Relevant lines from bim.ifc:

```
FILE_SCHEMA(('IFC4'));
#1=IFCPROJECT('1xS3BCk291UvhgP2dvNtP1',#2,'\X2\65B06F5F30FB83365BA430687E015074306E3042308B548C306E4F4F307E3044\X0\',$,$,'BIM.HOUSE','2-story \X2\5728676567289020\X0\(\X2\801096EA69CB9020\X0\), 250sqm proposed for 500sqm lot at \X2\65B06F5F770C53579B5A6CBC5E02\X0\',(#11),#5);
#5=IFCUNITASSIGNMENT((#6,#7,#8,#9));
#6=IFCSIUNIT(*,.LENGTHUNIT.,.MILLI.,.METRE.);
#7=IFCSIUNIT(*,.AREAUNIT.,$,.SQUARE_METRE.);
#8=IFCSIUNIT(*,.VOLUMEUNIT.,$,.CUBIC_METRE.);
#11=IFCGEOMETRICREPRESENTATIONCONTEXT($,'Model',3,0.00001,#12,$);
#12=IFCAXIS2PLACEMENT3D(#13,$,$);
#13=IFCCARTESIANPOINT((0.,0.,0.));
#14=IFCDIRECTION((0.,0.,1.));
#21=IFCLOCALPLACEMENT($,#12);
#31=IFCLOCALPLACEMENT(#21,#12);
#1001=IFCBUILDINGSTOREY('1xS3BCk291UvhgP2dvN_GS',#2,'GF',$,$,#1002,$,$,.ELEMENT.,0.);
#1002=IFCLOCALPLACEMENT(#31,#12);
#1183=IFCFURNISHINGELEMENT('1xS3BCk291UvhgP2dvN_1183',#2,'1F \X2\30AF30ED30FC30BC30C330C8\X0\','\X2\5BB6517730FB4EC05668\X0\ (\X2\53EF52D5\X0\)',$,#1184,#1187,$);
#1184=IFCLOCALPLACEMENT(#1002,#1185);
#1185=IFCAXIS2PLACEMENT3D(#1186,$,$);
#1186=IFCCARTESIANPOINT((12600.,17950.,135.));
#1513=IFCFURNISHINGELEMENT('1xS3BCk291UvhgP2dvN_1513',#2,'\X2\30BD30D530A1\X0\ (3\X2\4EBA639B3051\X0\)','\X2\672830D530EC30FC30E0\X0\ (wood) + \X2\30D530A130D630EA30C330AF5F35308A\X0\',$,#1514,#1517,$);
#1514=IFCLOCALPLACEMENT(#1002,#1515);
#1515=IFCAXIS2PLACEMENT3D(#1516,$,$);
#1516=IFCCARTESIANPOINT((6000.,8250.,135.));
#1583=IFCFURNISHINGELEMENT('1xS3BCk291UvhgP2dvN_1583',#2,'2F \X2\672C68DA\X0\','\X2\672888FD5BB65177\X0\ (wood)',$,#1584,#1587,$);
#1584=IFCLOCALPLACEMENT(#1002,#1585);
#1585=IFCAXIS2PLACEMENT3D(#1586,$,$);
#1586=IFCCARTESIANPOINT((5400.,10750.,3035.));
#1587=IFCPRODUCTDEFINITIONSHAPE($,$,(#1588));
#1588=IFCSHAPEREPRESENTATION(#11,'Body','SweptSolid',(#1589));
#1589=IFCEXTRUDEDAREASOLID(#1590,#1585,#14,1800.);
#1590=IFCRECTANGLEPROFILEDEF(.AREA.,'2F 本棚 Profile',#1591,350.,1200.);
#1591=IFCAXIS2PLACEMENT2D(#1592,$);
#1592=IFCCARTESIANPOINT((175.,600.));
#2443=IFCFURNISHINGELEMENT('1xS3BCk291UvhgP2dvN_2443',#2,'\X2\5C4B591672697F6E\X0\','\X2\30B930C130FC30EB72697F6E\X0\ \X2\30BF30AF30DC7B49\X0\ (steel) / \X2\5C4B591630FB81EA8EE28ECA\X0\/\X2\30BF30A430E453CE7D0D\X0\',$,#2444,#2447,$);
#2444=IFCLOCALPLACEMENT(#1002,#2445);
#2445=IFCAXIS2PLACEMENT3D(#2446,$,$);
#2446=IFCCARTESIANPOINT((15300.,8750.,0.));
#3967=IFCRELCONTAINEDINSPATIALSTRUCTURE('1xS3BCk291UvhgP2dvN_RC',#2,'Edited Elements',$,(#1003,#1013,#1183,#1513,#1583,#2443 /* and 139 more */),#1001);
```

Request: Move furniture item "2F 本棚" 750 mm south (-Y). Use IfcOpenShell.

```python
import ifcopenshell
import ifcopenshell.api.geometry
import ifcopenshell.util.placement
import ifcopenshell.util.unit

model = ifcopenshell.open("bim.ifc")
unit_scale = ifcopenshell.util.unit.calculate_unit_scale(model)

item = model.by_guid("1xS3BCk291UvhgP2dvN_1583")
matrix = ifcopenshell.util.placement.get_local_placement(item.ObjectPlacement)
matrix[1, 3] -= 0.75 / unit_scale
ifcopenshell.api.geometry.edit_object_placement(model, product=item, matrix=matrix, is_si=False)

print(ifcopenshell.util.placement.get_local_placement(item.ObjectPlacement).round(3) + 0.0)

model.write("bim_rev.ifc")
```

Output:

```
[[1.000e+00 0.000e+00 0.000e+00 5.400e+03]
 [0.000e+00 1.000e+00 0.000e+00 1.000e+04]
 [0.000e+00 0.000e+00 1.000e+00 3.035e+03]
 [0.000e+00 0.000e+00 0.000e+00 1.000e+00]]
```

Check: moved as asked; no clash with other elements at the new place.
